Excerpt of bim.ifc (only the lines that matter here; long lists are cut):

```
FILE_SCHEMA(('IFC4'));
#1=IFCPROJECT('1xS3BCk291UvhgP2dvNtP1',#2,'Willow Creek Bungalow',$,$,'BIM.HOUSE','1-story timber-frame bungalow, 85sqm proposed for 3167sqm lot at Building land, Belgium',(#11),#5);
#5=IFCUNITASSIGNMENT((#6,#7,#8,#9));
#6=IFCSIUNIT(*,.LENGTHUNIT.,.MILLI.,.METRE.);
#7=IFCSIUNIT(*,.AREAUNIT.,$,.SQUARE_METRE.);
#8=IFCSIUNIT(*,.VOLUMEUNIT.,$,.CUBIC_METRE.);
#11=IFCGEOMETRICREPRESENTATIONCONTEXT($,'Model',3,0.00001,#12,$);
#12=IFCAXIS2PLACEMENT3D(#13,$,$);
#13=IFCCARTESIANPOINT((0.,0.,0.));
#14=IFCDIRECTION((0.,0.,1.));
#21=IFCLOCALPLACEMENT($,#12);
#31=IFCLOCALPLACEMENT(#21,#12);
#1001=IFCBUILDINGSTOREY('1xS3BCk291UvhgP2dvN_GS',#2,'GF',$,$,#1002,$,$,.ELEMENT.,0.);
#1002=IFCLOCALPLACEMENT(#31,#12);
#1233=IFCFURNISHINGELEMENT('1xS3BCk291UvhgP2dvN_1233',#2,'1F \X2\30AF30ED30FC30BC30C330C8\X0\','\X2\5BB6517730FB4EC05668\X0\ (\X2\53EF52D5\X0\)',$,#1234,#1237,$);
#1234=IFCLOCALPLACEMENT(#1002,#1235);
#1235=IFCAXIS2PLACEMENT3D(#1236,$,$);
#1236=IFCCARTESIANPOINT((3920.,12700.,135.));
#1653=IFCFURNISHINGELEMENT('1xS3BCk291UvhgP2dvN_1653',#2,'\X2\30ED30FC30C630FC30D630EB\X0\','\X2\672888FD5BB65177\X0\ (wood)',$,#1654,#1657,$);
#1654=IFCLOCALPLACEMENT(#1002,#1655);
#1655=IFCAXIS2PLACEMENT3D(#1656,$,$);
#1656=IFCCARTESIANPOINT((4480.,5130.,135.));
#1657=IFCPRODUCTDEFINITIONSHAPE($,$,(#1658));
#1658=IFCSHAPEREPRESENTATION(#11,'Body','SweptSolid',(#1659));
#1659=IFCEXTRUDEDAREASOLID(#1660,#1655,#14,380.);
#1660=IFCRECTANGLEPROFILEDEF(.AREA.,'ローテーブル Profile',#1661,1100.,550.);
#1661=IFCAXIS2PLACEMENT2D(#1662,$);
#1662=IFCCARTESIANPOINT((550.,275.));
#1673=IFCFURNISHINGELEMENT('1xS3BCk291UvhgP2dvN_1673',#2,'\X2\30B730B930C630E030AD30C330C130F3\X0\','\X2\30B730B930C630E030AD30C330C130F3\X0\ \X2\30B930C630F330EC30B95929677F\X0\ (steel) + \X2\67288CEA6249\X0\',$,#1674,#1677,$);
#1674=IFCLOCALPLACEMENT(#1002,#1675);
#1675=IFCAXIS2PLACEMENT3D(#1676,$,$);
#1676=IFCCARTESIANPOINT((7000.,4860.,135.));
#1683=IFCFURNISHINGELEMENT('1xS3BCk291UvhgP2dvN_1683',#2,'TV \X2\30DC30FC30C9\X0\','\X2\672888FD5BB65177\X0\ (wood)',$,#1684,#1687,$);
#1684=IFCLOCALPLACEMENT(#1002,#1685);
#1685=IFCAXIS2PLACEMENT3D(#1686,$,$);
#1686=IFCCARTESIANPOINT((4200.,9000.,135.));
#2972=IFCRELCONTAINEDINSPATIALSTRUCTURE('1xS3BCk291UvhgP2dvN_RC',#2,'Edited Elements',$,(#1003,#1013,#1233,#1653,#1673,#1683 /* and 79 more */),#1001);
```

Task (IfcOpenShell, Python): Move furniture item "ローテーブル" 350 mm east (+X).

```python
import ifcopenshell
import ifcopenshell.api.geometry
import ifcopenshell.util.placement
import ifcopenshell.util.unit

model = ifcopenshell.open("bim.ifc")
unit_scale = ifcopenshell.util.unit.calculate_unit_scale(model)

item = model.by_guid("1xS3BCk291UvhgP2dvN_1653")
matrix = ifcopenshell.util.placement.get_local_placement(item.ObjectPlacement)
matrix[0, 3] += 0.35 / unit_scale
ifcopenshell.api.geometry.edit_object_placement(model, product=item, matrix=matrix, is_si=False)

print(ifcopenshell.util.placement.get_local_placement(item.ObjectPlacement).round(3) + 0.0)

model.write("bim_v2.ifc")
```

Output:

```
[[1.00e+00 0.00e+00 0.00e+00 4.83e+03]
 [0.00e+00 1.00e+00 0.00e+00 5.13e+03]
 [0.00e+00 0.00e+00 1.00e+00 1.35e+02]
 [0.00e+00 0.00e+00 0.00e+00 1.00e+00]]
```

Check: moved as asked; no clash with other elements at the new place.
